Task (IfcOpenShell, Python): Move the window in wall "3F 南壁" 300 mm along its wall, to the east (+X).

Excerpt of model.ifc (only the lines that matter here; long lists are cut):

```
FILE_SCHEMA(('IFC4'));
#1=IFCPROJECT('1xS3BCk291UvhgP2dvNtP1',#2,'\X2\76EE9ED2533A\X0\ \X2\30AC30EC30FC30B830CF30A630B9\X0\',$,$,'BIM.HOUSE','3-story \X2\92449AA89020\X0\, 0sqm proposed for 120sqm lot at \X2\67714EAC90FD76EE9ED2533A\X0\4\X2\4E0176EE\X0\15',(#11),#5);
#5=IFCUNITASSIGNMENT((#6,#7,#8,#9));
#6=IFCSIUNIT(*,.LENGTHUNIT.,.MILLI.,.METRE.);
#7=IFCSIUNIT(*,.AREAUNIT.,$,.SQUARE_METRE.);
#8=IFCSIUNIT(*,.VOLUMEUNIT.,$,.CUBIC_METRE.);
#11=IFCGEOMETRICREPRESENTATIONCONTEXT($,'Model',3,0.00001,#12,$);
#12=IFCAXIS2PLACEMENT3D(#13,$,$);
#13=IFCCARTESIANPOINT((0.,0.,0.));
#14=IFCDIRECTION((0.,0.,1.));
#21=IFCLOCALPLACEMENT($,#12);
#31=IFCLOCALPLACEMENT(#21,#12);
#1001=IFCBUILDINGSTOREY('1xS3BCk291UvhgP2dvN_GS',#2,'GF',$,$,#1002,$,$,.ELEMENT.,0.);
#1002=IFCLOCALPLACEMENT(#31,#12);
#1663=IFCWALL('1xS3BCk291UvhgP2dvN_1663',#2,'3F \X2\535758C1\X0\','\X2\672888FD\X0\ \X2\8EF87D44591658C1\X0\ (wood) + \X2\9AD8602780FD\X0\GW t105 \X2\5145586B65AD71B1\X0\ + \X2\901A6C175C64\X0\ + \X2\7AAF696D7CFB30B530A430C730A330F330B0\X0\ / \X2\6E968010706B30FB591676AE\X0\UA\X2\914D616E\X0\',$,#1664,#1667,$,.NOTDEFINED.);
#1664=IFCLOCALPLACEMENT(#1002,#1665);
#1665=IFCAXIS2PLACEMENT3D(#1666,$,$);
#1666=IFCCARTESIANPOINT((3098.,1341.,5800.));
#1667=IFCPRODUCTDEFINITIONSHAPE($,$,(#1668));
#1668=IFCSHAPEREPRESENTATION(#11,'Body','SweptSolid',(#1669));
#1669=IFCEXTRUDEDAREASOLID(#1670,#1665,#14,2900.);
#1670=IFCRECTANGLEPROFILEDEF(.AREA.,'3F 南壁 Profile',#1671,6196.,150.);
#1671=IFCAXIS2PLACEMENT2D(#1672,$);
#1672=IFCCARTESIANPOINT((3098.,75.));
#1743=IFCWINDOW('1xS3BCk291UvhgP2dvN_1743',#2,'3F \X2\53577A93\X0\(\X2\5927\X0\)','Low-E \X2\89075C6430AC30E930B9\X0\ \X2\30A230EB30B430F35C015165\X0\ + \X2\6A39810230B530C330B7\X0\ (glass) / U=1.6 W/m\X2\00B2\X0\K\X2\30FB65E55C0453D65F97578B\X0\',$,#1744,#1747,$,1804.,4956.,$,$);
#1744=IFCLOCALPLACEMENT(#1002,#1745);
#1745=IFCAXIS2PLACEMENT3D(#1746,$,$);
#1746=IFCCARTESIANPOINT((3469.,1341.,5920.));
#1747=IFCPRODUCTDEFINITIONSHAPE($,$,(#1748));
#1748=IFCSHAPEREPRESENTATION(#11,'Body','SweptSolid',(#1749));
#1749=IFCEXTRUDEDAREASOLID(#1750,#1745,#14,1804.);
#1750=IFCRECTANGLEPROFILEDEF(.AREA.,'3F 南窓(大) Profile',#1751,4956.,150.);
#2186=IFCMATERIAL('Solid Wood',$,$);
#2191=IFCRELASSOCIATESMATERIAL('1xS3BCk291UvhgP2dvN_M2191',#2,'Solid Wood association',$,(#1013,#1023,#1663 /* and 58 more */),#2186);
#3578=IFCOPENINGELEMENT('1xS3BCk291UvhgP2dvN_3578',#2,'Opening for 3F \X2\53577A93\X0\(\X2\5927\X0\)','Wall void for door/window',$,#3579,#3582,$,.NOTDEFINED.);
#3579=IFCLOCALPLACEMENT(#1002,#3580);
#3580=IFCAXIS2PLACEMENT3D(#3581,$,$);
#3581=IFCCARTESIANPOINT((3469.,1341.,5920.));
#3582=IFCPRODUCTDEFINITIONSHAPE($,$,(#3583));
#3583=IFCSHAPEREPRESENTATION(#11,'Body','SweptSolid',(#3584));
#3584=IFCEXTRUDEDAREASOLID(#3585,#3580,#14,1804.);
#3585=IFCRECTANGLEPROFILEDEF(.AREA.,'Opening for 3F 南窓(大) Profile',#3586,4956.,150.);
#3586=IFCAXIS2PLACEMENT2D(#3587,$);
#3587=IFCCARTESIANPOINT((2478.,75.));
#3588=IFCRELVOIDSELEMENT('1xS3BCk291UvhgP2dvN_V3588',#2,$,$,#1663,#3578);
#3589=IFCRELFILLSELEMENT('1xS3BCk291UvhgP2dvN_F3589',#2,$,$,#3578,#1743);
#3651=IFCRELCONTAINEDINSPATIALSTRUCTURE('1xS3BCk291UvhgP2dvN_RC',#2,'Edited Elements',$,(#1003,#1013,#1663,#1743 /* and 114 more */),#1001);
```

```python
import ifcopenshell
import ifcopenshell.api.geometry
import ifcopenshell.util.placement
import ifcopenshell.util.unit

model = ifcopenshell.open("model.ifc")
unit_scale = ifcopenshell.util.unit.calculate_unit_scale(model)

window = model.by_guid("1xS3BCk291UvhgP2dvN_1743")
opening = window.FillsVoids[0].RelatingOpeningElement
wall = opening.VoidsElements[0].RelatingBuildingElement

wall_matrix = ifcopenshell.util.placement.get_local_placement(wall.ObjectPlacement)
shift = wall_matrix[:3, 0] * 0.3 / unit_scale
before = ifcopenshell.util.placement.get_local_placement(window.ObjectPlacement)[:3, 3].copy()

# The window is not placed relative to its opening, so move both.
for product in (opening, window):
    matrix = ifcopenshell.util.placement.get_local_placement(product.ObjectPlacement)
    matrix[:3, 3] += shift
    ifcopenshell.api.geometry.edit_object_placement(model, product=product, matrix=matrix, is_si=False)

after = ifcopenshell.util.placement.get_local_placement(window.ObjectPlacement)[:3, 3]
print("window moved by", (after - before).round(3) + 0.0)

model.write("model_v2.ifc")
```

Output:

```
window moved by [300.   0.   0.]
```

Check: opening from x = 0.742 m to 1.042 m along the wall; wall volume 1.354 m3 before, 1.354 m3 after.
